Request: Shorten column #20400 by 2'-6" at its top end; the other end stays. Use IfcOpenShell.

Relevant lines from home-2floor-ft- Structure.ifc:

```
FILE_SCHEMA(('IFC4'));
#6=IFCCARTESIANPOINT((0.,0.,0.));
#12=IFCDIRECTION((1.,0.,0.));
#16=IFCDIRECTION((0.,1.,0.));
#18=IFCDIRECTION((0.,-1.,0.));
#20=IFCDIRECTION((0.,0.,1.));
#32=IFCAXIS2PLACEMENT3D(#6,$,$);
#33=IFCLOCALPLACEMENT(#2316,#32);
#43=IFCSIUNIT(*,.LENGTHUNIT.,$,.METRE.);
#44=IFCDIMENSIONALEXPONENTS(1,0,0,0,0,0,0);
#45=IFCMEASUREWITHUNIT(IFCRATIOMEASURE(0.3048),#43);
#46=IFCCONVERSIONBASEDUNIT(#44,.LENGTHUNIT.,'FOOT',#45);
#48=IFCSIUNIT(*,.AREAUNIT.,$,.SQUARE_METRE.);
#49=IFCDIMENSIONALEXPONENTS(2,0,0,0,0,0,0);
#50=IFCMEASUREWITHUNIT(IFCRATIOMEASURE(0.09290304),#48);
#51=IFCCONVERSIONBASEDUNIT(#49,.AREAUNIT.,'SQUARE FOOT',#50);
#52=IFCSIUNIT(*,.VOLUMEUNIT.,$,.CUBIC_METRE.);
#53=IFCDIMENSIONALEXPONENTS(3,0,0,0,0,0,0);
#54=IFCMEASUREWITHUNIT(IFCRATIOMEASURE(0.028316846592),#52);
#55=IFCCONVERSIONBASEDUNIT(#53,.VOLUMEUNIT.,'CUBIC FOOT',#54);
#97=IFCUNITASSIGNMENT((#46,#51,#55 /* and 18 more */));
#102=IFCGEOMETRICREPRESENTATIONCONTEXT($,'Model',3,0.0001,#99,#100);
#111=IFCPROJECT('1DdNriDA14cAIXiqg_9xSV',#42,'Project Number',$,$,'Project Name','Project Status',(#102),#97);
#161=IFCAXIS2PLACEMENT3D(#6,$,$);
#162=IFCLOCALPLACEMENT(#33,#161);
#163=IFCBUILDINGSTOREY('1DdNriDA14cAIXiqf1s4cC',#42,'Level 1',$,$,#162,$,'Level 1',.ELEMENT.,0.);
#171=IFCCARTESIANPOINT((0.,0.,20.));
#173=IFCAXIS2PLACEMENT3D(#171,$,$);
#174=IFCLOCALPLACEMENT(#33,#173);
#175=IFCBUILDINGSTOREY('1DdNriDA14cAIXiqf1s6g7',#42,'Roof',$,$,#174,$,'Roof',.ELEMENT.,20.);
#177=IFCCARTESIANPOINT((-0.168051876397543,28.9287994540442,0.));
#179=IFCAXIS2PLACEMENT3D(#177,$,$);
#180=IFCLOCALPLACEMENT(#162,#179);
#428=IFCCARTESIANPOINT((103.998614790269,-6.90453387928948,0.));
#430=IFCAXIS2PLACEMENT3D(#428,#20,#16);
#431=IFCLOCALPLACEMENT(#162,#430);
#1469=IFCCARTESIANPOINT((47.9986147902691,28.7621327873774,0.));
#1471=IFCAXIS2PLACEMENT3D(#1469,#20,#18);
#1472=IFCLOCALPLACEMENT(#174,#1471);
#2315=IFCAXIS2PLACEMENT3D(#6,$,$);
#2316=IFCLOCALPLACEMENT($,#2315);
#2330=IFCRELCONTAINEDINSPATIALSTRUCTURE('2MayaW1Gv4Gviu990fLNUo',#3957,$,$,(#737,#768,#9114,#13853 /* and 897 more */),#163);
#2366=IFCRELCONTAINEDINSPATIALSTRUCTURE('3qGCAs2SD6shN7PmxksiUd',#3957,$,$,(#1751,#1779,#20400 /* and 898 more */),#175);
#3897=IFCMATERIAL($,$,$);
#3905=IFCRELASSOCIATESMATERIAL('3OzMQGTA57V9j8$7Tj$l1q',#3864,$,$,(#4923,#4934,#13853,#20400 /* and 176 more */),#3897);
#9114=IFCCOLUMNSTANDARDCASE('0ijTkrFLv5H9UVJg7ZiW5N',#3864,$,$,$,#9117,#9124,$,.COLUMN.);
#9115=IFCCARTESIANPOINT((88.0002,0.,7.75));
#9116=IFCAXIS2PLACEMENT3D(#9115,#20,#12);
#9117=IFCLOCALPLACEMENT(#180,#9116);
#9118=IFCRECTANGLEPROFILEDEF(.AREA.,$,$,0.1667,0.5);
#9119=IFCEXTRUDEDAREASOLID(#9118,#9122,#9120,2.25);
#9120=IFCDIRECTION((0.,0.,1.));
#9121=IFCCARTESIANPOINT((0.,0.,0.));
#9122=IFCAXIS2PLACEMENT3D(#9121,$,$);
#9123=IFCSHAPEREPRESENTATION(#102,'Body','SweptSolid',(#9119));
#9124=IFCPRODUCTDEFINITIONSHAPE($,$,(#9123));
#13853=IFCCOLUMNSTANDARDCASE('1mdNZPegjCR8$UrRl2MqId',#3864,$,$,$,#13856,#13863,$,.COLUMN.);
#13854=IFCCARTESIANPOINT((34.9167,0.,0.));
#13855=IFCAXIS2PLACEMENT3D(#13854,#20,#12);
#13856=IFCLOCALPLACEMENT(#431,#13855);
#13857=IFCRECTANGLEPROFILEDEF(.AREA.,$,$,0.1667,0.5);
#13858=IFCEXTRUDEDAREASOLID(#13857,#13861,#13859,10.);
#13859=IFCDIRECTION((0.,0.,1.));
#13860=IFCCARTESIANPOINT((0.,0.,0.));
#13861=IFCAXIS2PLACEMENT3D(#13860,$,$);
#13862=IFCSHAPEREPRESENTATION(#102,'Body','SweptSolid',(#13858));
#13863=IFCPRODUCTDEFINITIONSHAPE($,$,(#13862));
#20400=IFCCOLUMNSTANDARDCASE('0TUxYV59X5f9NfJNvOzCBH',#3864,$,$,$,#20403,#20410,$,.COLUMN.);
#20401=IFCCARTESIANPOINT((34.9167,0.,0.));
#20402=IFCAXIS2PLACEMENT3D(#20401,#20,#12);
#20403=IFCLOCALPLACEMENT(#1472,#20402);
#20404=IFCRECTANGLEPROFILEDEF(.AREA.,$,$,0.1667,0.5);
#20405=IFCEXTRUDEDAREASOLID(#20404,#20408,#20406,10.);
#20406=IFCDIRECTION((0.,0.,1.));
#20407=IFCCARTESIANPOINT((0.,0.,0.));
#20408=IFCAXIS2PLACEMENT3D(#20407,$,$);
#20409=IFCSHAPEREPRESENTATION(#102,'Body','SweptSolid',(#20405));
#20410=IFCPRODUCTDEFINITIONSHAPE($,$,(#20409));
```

```python
import ifcopenshell
import ifcopenshell.util.unit

model = ifcopenshell.open("home-2floor-ft- Structure.ifc")
unit_scale = ifcopenshell.util.unit.calculate_unit_scale(model)

member = model.by_guid("0TUxYV59X5f9NfJNvOzCBH")
change = -30 * 0.0254 / unit_scale

# The extrusion runs towards the end named, so only its depth changes.
body = next(r for r in member.Representation.Representations if r.RepresentationIdentifier == "Body")
solid = body.Items[0]
old_length = solid.Depth
solid.Depth += change

print(f"length {old_length:g} -> {solid.Depth:g}")

model.write("home-2floor-ft- Structure_rev.ifc")
```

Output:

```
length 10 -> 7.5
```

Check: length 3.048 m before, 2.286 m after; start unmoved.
